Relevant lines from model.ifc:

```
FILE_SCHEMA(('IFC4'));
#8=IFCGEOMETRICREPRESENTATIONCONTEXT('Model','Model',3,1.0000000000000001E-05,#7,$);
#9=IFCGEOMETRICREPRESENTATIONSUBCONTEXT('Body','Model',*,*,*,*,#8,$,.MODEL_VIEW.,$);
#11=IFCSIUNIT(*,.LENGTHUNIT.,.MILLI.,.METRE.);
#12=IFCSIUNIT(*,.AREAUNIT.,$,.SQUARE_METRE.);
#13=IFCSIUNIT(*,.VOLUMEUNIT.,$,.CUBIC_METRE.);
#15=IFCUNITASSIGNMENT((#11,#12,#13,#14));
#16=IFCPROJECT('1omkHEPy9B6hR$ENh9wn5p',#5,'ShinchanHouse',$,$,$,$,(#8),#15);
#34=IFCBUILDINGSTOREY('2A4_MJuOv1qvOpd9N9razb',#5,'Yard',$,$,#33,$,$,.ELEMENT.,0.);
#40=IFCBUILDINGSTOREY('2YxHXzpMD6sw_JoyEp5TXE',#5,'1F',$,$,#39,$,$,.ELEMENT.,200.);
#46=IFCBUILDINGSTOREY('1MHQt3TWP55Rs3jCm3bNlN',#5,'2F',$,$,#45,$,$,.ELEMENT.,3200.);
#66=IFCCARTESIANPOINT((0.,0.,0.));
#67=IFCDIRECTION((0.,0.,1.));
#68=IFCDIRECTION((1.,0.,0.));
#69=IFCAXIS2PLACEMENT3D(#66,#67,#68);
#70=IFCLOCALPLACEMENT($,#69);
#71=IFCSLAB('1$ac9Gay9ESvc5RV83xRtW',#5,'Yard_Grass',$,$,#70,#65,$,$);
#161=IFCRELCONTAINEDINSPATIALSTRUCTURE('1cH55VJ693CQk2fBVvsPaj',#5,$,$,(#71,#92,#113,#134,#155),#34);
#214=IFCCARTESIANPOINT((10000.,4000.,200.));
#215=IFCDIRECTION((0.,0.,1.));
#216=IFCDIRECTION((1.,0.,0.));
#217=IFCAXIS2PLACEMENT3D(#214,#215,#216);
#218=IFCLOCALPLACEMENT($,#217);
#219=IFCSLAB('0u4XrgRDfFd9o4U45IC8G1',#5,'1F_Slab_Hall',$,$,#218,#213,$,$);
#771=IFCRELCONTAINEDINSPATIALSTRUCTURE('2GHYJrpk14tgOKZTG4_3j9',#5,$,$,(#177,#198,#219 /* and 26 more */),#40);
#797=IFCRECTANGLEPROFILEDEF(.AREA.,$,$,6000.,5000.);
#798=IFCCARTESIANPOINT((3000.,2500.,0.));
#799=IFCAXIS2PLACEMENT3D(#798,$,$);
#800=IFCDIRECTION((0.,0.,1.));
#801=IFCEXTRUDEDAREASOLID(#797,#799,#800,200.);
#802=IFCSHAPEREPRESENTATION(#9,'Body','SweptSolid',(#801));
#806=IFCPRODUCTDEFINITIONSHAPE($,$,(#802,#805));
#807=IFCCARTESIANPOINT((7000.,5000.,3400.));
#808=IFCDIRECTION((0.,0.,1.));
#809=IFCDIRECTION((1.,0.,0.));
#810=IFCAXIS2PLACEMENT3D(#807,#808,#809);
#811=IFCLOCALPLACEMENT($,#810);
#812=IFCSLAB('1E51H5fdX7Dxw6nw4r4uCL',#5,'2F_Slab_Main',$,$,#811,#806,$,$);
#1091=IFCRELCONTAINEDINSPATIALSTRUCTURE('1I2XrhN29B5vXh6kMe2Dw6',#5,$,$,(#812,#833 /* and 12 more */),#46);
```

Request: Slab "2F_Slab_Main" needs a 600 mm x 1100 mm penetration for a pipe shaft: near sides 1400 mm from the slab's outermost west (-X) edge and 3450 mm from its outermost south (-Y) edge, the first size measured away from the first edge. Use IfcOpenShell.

```python
import numpy as np
import ifcopenshell
import ifcopenshell.api.feature
import ifcopenshell.api.geometry
import ifcopenshell.api.root
import ifcopenshell.geom
import ifcopenshell.util.placement
import ifcopenshell.util.representation
import ifcopenshell.util.shape
import ifcopenshell.util.unit

model = ifcopenshell.open("model.ifc")
unit_scale = ifcopenshell.util.unit.calculate_unit_scale(model)
settings = ifcopenshell.geom.settings()


def volume(element):
    """Net volume in cubic metres, openings subtracted."""
    shape = ifcopenshell.geom.create_shape(settings, element)
    return ifcopenshell.util.shape.get_volume(shape.geometry)


slab = model.by_guid("1E51H5fdX7Dxw6nw4r4uCL")
before = volume(slab)

# Extent in the slab's own axes, in metres. The edges named are its -X and -Y sides.
slab_shape = ifcopenshell.geom.create_shape(settings, slab)
vertices = ifcopenshell.util.shape.get_vertices(slab_shape.geometry)
x_min, y_min, bottom = vertices.min(axis=0)
top = vertices[:, 2].max()

opening = ifcopenshell.api.root.create_entity(model, ifc_class="IfcOpeningElement", name="Pipe shaft opening", predefined_type="OPENING")
context = ifcopenshell.util.representation.get_context(model, "Model", "Body", "MODEL_VIEW")
width, depth = 0.6, 1.1
outline = [(0.0, 0.0), (width, 0.0), (width, depth), (0.0, depth), (0.0, 0.0)]
# Overshoot both faces by 50 mm so the cut is clean.
shape = ifcopenshell.api.geometry.add_slab_representation(
    model, context=context, depth=top - bottom + 0.1, polyline=outline
)
ifcopenshell.api.geometry.assign_representation(model, product=opening, representation=shape)

matrix = ifcopenshell.util.placement.get_local_placement(slab.ObjectPlacement)
matrix[:, 3] = matrix @ np.append(np.array([x_min + 1.4, y_min + 3.45, bottom - 0.05]) / unit_scale, 1.0)
ifcopenshell.api.geometry.edit_object_placement(model, product=opening, matrix=matrix, is_si=False)
ifcopenshell.api.feature.add_feature(model, feature=opening, element=slab)

after = volume(slab)

print(f"slab volume {before:.3f} -> {after:.3f} m3")

model.write("model_edited.ifc")
```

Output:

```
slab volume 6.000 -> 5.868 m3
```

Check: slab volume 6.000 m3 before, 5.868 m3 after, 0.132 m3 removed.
